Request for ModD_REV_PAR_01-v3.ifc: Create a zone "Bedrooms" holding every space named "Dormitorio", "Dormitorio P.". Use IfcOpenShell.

First a look at what the model holds.

```python
import ifcopenshell

model = ifcopenshell.open("ModD_REV_PAR_01-v3.ifc")
print(model.schema)
seen = {}
for space in model.by_type("IfcSpace"):
    seen[space.LongName] = seen.get(space.LongName, 0) + 1
for name, count in sorted(seen.items(), key=str):
    print(count, "x", name)
print("zones:", [z.Name for z in model.by_type("IfcZone")][:20])
```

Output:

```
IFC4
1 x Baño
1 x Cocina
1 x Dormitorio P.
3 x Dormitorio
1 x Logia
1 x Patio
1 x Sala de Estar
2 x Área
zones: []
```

```python
import ifcopenshell
import ifcopenshell.api.group
import ifcopenshell.api.root

model = ifcopenshell.open("ModD_REV_PAR_01-v3.ifc")

names = {"Dormitorio", "Dormitorio P."}
spaces = [s for s in model.by_type("IfcSpace") if s.LongName in names]

zone = ifcopenshell.api.root.create_entity(model, ifc_class="IfcZone", name="Bedrooms")
ifcopenshell.api.group.assign_group(model, products=spaces, group=zone)
print(len(spaces), "spaces in", zone.Name)

model.write("ModD_REV_PAR_01-v3_rev.ifc")
```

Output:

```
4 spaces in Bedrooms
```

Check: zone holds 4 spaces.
